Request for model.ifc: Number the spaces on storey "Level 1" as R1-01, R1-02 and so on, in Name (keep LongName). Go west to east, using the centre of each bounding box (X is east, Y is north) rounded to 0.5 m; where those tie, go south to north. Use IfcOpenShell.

First a look at what the model holds.

```python
import ifcopenshell
import ifcopenshell.util.element
import ifcopenshell.util.placement

model = ifcopenshell.open("model.ifc")
print(model.schema)
storey = next(s for s in model.by_type("IfcBuildingStorey") if s.Name == "Level 1")
spaces = [e for e in ifcopenshell.util.element.get_decomposition(storey) if e.is_a("IfcSpace")]
for e in sorted(spaces, key=lambda e: e.id()):
    origin = ifcopenshell.util.placement.get_local_placement(e.ObjectPlacement)[:3, 3]
    print(e.id(), e.Name, e.LongName, origin.round(2) + 0.0, sep=" | ")
```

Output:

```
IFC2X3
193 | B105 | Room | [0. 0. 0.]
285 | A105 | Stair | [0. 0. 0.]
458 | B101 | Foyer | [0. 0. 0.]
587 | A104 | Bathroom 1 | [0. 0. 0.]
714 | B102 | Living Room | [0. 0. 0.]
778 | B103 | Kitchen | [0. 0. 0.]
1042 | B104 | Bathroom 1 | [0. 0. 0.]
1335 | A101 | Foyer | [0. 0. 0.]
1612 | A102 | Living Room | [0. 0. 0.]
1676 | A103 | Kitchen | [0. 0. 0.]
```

```python
import ifcopenshell
import ifcopenshell.geom
import ifcopenshell.util.element
import ifcopenshell.util.shape

model = ifcopenshell.open("model.ifc")
settings = ifcopenshell.geom.settings()
settings.set("use-world-coords", True)


def centre(element):
    shape = ifcopenshell.geom.create_shape(settings, element)
    return ifcopenshell.util.shape.get_bbox_centroid(shape.geometry)


storey = next(s for s in model.by_type("IfcBuildingStorey") if s.Name == "Level 1")
spaces = [e for e in ifcopenshell.util.element.get_decomposition(storey) if e.is_a("IfcSpace")]

# Insertion points can sit at a corner or the storey origin, so sort by the geometry (in metres).
centres = {e: centre(e) for e in spaces}
spaces.sort(key=lambda e: (round(centres[e][0] / 0.5), centres[e][1]))

for i, e in enumerate(spaces, start=1):
    number = f"R1-{i:02d}"
    e.Name = number
    print(e.id(), number)

model.write("model_edited.ifc")
```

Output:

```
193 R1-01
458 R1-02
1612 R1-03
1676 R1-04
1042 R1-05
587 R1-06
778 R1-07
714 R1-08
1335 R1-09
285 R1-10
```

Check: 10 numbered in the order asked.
